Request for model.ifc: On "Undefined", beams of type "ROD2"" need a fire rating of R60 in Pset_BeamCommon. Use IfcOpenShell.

First a look at what the model holds.

```python
import ifcopenshell
import ifcopenshell.util.element

model = ifcopenshell.open("model.ifc")
print(model.schema)
storey = next(s for s in model.by_type("IfcBuildingStorey") if s.Name == "Undefined")
beams = [e for e in ifcopenshell.util.element.get_decomposition(storey) if e.is_a("IfcBeam")]
seen = {}
for e in beams:
    element_type = ifcopenshell.util.element.get_type(e)
    key = (element_type.Name if element_type != e and element_type else None, ifcopenshell.util.element.get_pset(e, "Pset_BeamCommon", "FireRating"))
    seen[key] = seen.get(key, 0) + 1
for (name, value), count in sorted(seen.items(), key=str):
    print(count, "x", name, "|", value)
```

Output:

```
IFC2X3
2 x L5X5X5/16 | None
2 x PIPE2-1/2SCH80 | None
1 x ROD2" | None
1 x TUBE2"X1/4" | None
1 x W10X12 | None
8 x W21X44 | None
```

```python
import ifcopenshell
import ifcopenshell.api.pset
import ifcopenshell.util.element

model = ifcopenshell.open("model.ifc")

storey = next(s for s in model.by_type("IfcBuildingStorey") if s.Name == "Undefined")
beams = [e for e in ifcopenshell.util.element.get_decomposition(storey) if e.is_a("IfcBeam")]

count = 0
for e in beams:
    element_type = ifcopenshell.util.element.get_type(e)
    if element_type in (None, e) or element_type.Name != 'ROD2"':
        continue
    # add_pset returns the element's existing set when there is one.
    pset = ifcopenshell.api.pset.add_pset(model, product=e, name="Pset_BeamCommon")
    ifcopenshell.api.pset.edit_pset(model, pset=pset, properties={"FireRating": "R60"})
    count += 1

print(count, "beams updated")

model.write("model-out.ifc")
```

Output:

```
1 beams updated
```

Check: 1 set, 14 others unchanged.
